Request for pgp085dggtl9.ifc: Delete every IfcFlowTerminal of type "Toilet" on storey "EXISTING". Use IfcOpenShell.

First a look at what the model holds.

```python
import ifcopenshell
import ifcopenshell.util.element

model = ifcopenshell.open("pgp085dggtl9.ifc")
print(model.schema)
storey = next(s for s in model.by_type("IfcBuildingStorey") if s.Name == "EXISTING")
terminals = [e for e in ifcopenshell.util.element.get_decomposition(storey) if e.is_a("IfcFlowTerminal")]
seen = {}
for e in terminals:
    element_type = ifcopenshell.util.element.get_type(e)
    name = element_type.Name if element_type not in (None, e) else None
    seen[name] = seen.get(name, 0) + 1
for name, count in sorted(seen.items(), key=str):
    print(count, "x", name)
```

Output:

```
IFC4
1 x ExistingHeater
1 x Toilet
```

```python
import ifcopenshell
import ifcopenshell.api.root
import ifcopenshell.util.element

model = ifcopenshell.open("pgp085dggtl9.ifc")

storey = next(s for s in model.by_type("IfcBuildingStorey") if s.Name == "EXISTING")
terminals = [e for e in ifcopenshell.util.element.get_decomposition(storey) if e.is_a("IfcFlowTerminal")]
targets = [e for e in terminals if (t := ifcopenshell.util.element.get_type(e)) not in (None, e) and t.Name == "Toilet"]

for e in targets:
    ifcopenshell.api.root.remove_product(model, product=e)
print(len(targets), "removed")

model.write("pgp085dggtl9_updated.ifc")
```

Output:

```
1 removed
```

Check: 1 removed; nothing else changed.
